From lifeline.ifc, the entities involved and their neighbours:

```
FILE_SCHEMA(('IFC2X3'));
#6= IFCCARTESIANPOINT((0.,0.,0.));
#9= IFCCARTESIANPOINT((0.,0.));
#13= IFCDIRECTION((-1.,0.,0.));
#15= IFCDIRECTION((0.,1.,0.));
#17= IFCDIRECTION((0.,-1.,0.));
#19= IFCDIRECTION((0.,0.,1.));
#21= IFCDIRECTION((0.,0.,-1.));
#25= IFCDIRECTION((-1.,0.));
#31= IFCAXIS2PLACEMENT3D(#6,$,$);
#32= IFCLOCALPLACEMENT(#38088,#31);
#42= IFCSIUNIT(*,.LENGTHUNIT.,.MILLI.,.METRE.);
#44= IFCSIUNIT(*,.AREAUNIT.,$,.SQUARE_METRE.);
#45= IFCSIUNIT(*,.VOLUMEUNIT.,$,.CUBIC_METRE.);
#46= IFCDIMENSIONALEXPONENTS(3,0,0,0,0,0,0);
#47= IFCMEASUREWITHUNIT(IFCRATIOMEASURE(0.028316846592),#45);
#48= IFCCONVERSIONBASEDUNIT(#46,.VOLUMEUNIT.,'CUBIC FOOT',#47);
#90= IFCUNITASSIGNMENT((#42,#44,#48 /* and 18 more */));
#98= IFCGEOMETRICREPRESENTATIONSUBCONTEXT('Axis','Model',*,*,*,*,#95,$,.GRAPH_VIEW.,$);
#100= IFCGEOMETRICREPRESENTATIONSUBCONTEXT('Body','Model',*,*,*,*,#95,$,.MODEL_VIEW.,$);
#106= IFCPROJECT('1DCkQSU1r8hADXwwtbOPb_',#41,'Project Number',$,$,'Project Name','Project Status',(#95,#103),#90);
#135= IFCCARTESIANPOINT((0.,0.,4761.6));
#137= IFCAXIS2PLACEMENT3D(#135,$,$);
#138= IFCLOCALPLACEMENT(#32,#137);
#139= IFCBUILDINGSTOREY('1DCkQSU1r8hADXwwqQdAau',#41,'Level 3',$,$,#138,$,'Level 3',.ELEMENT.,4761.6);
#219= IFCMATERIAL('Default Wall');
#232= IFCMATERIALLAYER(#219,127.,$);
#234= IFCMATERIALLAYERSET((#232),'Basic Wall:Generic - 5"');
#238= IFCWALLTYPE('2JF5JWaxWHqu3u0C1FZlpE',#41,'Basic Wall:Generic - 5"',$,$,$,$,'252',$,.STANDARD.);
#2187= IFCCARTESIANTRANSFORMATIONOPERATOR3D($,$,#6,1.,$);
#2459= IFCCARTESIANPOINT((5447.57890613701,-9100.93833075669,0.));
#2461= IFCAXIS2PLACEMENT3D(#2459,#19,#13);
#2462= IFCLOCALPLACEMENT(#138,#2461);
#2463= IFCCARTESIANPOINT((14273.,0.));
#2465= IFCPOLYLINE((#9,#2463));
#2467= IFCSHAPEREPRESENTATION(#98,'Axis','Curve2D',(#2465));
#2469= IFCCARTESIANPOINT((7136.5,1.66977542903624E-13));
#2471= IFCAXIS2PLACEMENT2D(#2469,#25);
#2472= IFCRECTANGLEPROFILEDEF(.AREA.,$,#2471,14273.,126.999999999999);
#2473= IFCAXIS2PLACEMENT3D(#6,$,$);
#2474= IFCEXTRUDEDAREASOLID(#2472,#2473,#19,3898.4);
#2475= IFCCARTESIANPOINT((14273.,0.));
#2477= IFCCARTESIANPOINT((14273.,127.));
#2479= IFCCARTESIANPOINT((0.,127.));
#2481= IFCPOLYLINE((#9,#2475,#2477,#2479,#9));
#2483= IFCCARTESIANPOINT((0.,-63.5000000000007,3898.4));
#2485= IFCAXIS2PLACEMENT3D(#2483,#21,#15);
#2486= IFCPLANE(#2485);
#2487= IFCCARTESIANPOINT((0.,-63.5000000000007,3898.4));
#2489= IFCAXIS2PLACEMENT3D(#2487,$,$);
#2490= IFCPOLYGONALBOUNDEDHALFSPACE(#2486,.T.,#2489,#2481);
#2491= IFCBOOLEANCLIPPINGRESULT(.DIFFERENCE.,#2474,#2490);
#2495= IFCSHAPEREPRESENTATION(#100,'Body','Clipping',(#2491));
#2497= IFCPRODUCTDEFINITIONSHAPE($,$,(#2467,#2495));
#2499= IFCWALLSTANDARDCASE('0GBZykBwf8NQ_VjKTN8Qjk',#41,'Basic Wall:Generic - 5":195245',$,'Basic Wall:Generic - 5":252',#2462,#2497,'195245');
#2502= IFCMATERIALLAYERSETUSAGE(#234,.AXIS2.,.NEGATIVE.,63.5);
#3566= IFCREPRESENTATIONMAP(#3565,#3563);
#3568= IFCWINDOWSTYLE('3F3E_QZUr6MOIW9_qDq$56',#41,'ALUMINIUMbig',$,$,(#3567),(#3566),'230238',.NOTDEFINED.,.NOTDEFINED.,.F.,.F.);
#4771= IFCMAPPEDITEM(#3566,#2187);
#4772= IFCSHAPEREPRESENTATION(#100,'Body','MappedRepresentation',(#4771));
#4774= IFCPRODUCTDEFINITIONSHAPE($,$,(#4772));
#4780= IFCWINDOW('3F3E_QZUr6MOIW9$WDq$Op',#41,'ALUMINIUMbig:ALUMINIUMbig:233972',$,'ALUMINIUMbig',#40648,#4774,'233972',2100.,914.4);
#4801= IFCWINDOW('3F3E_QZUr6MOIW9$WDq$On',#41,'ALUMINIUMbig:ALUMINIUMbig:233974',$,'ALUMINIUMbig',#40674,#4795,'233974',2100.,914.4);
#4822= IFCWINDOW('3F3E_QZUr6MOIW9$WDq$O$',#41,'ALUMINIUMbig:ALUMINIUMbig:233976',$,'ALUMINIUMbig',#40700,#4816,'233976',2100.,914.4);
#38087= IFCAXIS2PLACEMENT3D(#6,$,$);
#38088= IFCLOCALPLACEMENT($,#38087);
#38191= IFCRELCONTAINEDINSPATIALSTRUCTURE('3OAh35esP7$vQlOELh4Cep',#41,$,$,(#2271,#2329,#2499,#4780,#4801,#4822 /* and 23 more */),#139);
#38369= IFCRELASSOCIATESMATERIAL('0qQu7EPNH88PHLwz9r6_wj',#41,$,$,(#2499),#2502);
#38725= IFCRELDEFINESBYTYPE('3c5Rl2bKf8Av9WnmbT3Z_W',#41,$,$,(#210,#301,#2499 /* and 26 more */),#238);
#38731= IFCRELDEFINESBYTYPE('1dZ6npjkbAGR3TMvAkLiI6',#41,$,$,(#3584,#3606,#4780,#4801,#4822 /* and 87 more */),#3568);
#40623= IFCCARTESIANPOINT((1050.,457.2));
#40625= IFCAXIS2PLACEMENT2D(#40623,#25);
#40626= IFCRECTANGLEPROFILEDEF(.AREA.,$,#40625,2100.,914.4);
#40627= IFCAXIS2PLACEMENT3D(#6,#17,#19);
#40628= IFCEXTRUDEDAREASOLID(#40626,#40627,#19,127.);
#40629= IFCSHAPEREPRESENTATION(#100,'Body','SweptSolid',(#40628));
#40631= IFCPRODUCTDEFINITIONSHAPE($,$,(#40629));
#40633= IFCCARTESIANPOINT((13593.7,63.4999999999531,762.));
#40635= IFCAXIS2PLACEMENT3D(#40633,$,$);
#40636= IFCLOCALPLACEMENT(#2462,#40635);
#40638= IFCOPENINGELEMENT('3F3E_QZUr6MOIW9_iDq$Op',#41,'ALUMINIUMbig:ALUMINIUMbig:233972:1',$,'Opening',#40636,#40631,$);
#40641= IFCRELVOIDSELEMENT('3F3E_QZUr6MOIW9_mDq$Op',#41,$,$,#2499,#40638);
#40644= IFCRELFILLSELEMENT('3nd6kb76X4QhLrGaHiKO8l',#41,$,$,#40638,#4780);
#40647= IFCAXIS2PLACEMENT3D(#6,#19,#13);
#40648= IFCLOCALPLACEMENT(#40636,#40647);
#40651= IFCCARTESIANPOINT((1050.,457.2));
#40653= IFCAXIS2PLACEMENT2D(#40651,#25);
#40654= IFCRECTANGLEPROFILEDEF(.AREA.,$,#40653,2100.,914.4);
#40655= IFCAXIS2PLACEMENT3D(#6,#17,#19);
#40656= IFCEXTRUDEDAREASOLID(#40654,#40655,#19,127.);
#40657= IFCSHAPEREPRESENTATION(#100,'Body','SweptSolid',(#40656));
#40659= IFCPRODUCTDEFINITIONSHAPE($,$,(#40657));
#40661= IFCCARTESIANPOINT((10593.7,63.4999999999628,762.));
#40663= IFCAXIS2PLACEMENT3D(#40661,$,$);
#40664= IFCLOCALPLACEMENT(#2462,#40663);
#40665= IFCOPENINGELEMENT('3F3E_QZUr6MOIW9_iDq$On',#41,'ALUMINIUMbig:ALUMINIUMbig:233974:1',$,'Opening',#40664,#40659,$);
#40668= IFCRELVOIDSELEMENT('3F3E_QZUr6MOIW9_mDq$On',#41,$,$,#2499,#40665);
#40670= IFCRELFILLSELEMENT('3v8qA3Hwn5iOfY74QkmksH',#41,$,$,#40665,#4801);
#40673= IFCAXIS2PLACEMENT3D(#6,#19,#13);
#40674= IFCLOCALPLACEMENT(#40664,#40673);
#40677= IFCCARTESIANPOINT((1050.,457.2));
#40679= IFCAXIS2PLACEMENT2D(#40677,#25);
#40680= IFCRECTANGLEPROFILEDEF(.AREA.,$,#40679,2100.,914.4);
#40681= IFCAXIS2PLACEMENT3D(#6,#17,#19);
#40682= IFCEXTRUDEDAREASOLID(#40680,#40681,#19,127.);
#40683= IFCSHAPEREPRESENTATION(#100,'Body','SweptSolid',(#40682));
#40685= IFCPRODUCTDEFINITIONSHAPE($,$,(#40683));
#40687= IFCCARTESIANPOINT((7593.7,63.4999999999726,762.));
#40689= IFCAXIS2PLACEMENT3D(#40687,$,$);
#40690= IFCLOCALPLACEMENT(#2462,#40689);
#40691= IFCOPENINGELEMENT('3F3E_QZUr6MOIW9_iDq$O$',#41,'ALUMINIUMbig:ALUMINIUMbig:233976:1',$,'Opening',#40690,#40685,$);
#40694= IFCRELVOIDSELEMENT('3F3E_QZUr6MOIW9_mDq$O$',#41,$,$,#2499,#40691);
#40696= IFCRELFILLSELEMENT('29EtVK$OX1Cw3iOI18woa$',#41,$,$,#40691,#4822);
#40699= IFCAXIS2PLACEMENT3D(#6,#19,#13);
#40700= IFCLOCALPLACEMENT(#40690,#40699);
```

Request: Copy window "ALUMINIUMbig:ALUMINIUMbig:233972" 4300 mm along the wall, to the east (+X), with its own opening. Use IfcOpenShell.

```python
import ifcopenshell
import ifcopenshell.api.feature
import ifcopenshell.api.geometry
import ifcopenshell.api.root
import ifcopenshell.geom
import ifcopenshell.util.element
import ifcopenshell.util.placement
import ifcopenshell.util.shape
import ifcopenshell.util.unit

model = ifcopenshell.open("lifeline.ifc")
unit_scale = ifcopenshell.util.unit.calculate_unit_scale(model)
settings = ifcopenshell.geom.settings()


def volume(element):
    """Net volume in cubic metres, openings subtracted."""
    shape = ifcopenshell.geom.create_shape(settings, element)
    return ifcopenshell.util.shape.get_volume(shape.geometry)


def reuse_history(source, copy):
    """copy_class also copies each property set's owner history, people and application; keep the originals."""
    for rel in copy.IsDefinedBy:
        if rel.is_a("IfcRelDefinesByProperties") and (history := rel.RelatingPropertyDefinition.OwnerHistory):
            rel.RelatingPropertyDefinition.OwnerHistory = source.OwnerHistory
            ifcopenshell.util.element.remove_deep2(model, history)


window = model.by_guid("3F3E_QZUr6MOIW9$WDq$Op")
opening = window.FillsVoids[0].RelatingOpeningElement
wall = opening.VoidsElements[0].RelatingBuildingElement
before = volume(wall)
shift = ifcopenshell.util.placement.get_local_placement(wall.ObjectPlacement)[:3, 0] * -4.3 / unit_scale

# copy_class copies the void relationship, type, container and properties, but no geometry.
new_opening = ifcopenshell.api.root.copy_class(model, product=opening)
new_opening.Representation = ifcopenshell.util.element.copy_deep(
    model, opening.Representation, exclude=["IfcGeometricRepresentationContext", "IfcRepresentationMap"]
)
new_opening.Name = "ALUMINIUMbig:ALUMINIUMbig"
new_window = ifcopenshell.api.root.copy_class(model, product=window)
new_window.Representation = ifcopenshell.util.element.copy_deep(
    model, window.Representation, exclude=["IfcGeometricRepresentationContext", "IfcRepresentationMap"]
)
new_window.Name = "ALUMINIUMbig:ALUMINIUMbig"
new_window.Tag = None
reuse_history(window, new_window)
fills = ifcopenshell.api.feature.add_filling(model, opening=new_opening, element=new_window)
fills.OwnerHistory = new_window.OwnerHistory  # required in IFC2X3

for old, new in ((opening, new_opening), (window, new_window)):
    matrix = ifcopenshell.util.placement.get_local_placement(old.ObjectPlacement)
    matrix[:3, 3] += shift
    ifcopenshell.api.geometry.edit_object_placement(model, product=new, matrix=matrix, is_si=False)

after = volume(wall)

print(f"wall volume {before:.3f} -> {after:.3f} m3")

model.write("lifeline_updated.ifc")
```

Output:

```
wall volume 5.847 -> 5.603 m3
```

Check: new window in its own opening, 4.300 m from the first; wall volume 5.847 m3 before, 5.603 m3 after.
